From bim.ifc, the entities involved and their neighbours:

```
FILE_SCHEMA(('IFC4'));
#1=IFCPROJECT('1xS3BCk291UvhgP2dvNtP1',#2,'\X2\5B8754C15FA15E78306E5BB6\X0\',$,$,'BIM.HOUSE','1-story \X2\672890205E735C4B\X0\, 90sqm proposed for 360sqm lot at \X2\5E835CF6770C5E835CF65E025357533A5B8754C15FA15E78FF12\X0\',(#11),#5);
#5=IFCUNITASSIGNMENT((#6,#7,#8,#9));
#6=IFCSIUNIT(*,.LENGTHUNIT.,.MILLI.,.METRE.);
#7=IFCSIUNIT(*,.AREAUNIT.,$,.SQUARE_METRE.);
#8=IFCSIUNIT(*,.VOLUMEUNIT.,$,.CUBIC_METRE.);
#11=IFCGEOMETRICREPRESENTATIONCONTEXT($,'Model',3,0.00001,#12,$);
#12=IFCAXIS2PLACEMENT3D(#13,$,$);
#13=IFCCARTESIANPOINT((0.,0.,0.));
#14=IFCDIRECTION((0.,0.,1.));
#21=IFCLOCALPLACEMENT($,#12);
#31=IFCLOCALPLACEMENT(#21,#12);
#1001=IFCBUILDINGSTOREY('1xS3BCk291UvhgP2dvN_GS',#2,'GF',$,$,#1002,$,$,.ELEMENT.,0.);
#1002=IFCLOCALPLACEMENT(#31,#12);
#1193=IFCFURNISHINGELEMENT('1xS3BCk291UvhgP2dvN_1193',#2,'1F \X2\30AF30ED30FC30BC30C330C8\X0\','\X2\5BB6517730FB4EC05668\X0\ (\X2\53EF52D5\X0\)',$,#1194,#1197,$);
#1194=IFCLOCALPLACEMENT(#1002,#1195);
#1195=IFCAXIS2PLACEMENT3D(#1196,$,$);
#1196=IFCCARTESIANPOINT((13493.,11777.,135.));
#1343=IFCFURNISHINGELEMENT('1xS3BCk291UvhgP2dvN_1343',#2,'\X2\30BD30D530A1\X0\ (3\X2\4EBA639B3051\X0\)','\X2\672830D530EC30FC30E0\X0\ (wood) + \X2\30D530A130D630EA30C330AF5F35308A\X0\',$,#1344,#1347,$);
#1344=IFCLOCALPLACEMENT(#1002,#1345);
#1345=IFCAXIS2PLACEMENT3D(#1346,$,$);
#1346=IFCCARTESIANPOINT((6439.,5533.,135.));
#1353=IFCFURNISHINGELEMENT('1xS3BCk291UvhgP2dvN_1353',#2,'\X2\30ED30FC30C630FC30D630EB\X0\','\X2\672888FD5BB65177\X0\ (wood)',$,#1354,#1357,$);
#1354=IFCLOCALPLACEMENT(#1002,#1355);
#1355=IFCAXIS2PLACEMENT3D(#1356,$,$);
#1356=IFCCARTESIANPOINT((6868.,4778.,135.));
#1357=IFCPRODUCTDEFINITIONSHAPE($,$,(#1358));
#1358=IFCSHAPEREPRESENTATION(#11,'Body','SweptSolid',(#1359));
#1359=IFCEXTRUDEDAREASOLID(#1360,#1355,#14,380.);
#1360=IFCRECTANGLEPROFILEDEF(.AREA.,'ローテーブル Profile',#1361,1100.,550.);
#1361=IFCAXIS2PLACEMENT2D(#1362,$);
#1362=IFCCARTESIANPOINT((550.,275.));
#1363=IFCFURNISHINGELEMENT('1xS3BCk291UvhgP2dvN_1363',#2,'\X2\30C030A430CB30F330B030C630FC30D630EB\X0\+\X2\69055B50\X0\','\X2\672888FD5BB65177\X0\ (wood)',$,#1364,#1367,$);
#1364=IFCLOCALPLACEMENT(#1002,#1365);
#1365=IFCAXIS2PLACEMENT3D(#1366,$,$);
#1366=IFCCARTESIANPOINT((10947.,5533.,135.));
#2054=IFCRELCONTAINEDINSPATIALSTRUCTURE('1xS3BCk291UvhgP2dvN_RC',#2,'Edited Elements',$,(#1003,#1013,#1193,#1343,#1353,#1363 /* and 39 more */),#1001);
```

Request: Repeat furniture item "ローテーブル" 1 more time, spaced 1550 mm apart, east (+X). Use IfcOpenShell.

```python
import numpy as np
import ifcopenshell
import ifcopenshell.api.geometry
import ifcopenshell.api.root
import ifcopenshell.util.element
import ifcopenshell.util.placement
import ifcopenshell.util.unit

model = ifcopenshell.open("bim.ifc")
unit_scale = ifcopenshell.util.unit.calculate_unit_scale(model)


def reuse_history(source, copy):
    """copy_class also copies each property set's owner history, people and application; keep the originals."""
    for rel in copy.IsDefinedBy:
        if rel.is_a("IfcRelDefinesByProperties") and (history := rel.RelatingPropertyDefinition.OwnerHistory):
            rel.RelatingPropertyDefinition.OwnerHistory = source.OwnerHistory
            ifcopenshell.util.element.remove_deep2(model, history)


source = model.by_guid("1xS3BCk291UvhgP2dvN_1353")
base = ifcopenshell.util.placement.get_local_placement(source.ObjectPlacement)
step = np.array([1.0, 0.0, 0.0]) * 1.55 / unit_scale

for i in range(1, 2):
    copy = ifcopenshell.api.root.copy_class(model, product=source)
    copy.Representation = ifcopenshell.util.element.copy_deep(
        model, source.Representation, exclude=["IfcGeometricRepresentationContext", "IfcRepresentationMap"]
    )
    reuse_history(source, copy)
    matrix = base.copy()
    matrix[:3, 3] += i * step
    print("added at", matrix[:3, 3].round(3) + 0.0)
    ifcopenshell.api.geometry.edit_object_placement(model, product=copy, matrix=matrix, is_si=False)

model.write("bim_updated.ifc")
```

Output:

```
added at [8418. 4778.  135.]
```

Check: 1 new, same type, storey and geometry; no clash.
